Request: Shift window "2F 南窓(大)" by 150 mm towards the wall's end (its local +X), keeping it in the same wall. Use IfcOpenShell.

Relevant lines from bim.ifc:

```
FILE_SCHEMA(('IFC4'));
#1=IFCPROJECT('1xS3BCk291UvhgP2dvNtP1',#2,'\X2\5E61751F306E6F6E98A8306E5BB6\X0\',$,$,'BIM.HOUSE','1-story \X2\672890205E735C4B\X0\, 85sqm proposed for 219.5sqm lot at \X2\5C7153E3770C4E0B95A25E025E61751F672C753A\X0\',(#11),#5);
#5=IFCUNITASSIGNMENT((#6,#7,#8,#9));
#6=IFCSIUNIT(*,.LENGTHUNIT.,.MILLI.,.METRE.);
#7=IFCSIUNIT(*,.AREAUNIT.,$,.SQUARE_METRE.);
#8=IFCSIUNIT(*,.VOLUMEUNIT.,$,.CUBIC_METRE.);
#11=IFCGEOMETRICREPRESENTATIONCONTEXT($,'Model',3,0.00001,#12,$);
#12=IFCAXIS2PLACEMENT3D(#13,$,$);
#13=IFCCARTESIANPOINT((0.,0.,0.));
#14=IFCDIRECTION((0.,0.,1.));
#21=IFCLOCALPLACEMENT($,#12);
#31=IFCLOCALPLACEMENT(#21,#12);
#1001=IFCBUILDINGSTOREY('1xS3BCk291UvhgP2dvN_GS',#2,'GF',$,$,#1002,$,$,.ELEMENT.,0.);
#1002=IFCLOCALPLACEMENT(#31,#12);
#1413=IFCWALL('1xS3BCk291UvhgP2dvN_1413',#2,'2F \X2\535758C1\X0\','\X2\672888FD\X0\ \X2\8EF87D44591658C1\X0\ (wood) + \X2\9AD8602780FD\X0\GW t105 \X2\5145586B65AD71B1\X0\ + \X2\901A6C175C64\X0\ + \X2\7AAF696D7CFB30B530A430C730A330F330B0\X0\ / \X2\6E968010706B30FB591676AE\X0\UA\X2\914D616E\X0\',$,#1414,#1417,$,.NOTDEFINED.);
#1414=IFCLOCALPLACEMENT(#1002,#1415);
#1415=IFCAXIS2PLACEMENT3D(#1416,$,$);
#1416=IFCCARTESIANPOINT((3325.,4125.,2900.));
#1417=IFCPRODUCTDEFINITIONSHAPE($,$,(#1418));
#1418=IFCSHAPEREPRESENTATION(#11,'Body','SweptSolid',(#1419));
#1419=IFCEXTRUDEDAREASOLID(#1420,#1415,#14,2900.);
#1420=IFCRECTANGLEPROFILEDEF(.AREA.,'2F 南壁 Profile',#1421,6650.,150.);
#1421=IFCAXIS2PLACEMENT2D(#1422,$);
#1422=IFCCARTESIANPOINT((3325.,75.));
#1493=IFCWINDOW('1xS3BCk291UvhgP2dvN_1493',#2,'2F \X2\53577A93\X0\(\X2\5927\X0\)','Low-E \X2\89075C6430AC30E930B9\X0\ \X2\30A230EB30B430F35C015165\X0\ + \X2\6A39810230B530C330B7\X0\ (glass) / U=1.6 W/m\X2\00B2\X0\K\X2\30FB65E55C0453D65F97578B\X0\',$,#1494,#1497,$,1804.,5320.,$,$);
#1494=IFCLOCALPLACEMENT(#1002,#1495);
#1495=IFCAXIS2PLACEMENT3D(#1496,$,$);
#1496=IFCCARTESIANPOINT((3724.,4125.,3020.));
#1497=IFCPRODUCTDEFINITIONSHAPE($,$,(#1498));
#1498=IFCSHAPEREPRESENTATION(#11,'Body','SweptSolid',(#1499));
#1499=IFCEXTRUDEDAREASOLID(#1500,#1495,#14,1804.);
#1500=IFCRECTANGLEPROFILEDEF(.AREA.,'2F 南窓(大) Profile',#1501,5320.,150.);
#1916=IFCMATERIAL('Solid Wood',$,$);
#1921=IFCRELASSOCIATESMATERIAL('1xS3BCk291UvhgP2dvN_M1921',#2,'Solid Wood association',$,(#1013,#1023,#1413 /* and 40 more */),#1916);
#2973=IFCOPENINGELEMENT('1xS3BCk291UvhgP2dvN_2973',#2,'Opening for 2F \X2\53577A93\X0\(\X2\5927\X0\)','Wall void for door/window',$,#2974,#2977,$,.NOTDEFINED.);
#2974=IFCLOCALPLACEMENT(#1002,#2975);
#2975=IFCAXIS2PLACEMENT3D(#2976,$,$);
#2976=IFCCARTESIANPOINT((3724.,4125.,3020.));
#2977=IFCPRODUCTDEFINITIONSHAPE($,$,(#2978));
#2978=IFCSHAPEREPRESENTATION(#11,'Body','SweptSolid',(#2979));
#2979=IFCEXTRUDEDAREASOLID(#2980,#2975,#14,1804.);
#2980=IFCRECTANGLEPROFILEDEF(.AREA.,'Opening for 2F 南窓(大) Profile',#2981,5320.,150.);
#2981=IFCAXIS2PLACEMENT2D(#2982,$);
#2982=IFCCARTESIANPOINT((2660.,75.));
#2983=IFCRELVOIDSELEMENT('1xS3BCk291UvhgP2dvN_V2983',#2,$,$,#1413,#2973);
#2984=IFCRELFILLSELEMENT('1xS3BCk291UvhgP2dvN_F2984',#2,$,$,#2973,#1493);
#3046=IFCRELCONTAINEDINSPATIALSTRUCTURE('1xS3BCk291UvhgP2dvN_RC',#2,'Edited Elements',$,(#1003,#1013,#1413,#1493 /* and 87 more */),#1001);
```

```python
import ifcopenshell
import ifcopenshell.api.geometry
import ifcopenshell.util.placement

model = ifcopenshell.open("bim.ifc")

window = model.by_guid("1xS3BCk291UvhgP2dvN_1493")
opening = window.FillsVoids[0].RelatingOpeningElement
wall = opening.VoidsElements[0].RelatingBuildingElement

wall_matrix = ifcopenshell.util.placement.get_local_placement(wall.ObjectPlacement)
shift = wall_matrix[:3, 0] * 150.0
before = ifcopenshell.util.placement.get_local_placement(window.ObjectPlacement)[:3, 3].copy()

# The window is not placed relative to its opening, so move both.
for product in (opening, window):
    matrix = ifcopenshell.util.placement.get_local_placement(product.ObjectPlacement)
    matrix[:3, 3] += shift
    ifcopenshell.api.geometry.edit_object_placement(model, product=product, matrix=matrix, is_si=False)

after = ifcopenshell.util.placement.get_local_placement(window.ObjectPlacement)[:3, 3]
print("window moved by", (after - before).round(3) + 0.0)

model.write("bim-out.ifc")
```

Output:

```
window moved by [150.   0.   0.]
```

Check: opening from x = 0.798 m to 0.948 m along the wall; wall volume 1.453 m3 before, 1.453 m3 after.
